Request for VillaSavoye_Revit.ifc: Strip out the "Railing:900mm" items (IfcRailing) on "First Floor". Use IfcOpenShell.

First a look at what the model holds.

```python
import ifcopenshell
import ifcopenshell.util.element

model = ifcopenshell.open("VillaSavoye_Revit.ifc")
print(model.schema)
storey = next(s for s in model.by_type("IfcBuildingStorey") if s.Name == "First Floor")
railings = [e for e in ifcopenshell.util.element.get_decomposition(storey) if e.is_a("IfcRailing")]
seen = {}
for e in railings:
    element_type = ifcopenshell.util.element.get_type(e)
    name = element_type.Name if element_type not in (None, e) else None
    seen[name] = seen.get(name, 0) + 1
for name, count in sorted(seen.items(), key=str):
    print(count, "x", name)
```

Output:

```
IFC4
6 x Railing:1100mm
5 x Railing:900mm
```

```python
import ifcopenshell
import ifcopenshell.api.root
import ifcopenshell.util.element

model = ifcopenshell.open("VillaSavoye_Revit.ifc")

storey = next(s for s in model.by_type("IfcBuildingStorey") if s.Name == "First Floor")
railings = [e for e in ifcopenshell.util.element.get_decomposition(storey) if e.is_a("IfcRailing")]
targets = [e for e in railings if (t := ifcopenshell.util.element.get_type(e)) not in (None, e) and t.Name == "Railing:900mm"]

for e in targets:
    ifcopenshell.api.root.remove_product(model, product=e)
print(len(targets), "removed")

model.write("VillaSavoye_Revit-out.ifc")
```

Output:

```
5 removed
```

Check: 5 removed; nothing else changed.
